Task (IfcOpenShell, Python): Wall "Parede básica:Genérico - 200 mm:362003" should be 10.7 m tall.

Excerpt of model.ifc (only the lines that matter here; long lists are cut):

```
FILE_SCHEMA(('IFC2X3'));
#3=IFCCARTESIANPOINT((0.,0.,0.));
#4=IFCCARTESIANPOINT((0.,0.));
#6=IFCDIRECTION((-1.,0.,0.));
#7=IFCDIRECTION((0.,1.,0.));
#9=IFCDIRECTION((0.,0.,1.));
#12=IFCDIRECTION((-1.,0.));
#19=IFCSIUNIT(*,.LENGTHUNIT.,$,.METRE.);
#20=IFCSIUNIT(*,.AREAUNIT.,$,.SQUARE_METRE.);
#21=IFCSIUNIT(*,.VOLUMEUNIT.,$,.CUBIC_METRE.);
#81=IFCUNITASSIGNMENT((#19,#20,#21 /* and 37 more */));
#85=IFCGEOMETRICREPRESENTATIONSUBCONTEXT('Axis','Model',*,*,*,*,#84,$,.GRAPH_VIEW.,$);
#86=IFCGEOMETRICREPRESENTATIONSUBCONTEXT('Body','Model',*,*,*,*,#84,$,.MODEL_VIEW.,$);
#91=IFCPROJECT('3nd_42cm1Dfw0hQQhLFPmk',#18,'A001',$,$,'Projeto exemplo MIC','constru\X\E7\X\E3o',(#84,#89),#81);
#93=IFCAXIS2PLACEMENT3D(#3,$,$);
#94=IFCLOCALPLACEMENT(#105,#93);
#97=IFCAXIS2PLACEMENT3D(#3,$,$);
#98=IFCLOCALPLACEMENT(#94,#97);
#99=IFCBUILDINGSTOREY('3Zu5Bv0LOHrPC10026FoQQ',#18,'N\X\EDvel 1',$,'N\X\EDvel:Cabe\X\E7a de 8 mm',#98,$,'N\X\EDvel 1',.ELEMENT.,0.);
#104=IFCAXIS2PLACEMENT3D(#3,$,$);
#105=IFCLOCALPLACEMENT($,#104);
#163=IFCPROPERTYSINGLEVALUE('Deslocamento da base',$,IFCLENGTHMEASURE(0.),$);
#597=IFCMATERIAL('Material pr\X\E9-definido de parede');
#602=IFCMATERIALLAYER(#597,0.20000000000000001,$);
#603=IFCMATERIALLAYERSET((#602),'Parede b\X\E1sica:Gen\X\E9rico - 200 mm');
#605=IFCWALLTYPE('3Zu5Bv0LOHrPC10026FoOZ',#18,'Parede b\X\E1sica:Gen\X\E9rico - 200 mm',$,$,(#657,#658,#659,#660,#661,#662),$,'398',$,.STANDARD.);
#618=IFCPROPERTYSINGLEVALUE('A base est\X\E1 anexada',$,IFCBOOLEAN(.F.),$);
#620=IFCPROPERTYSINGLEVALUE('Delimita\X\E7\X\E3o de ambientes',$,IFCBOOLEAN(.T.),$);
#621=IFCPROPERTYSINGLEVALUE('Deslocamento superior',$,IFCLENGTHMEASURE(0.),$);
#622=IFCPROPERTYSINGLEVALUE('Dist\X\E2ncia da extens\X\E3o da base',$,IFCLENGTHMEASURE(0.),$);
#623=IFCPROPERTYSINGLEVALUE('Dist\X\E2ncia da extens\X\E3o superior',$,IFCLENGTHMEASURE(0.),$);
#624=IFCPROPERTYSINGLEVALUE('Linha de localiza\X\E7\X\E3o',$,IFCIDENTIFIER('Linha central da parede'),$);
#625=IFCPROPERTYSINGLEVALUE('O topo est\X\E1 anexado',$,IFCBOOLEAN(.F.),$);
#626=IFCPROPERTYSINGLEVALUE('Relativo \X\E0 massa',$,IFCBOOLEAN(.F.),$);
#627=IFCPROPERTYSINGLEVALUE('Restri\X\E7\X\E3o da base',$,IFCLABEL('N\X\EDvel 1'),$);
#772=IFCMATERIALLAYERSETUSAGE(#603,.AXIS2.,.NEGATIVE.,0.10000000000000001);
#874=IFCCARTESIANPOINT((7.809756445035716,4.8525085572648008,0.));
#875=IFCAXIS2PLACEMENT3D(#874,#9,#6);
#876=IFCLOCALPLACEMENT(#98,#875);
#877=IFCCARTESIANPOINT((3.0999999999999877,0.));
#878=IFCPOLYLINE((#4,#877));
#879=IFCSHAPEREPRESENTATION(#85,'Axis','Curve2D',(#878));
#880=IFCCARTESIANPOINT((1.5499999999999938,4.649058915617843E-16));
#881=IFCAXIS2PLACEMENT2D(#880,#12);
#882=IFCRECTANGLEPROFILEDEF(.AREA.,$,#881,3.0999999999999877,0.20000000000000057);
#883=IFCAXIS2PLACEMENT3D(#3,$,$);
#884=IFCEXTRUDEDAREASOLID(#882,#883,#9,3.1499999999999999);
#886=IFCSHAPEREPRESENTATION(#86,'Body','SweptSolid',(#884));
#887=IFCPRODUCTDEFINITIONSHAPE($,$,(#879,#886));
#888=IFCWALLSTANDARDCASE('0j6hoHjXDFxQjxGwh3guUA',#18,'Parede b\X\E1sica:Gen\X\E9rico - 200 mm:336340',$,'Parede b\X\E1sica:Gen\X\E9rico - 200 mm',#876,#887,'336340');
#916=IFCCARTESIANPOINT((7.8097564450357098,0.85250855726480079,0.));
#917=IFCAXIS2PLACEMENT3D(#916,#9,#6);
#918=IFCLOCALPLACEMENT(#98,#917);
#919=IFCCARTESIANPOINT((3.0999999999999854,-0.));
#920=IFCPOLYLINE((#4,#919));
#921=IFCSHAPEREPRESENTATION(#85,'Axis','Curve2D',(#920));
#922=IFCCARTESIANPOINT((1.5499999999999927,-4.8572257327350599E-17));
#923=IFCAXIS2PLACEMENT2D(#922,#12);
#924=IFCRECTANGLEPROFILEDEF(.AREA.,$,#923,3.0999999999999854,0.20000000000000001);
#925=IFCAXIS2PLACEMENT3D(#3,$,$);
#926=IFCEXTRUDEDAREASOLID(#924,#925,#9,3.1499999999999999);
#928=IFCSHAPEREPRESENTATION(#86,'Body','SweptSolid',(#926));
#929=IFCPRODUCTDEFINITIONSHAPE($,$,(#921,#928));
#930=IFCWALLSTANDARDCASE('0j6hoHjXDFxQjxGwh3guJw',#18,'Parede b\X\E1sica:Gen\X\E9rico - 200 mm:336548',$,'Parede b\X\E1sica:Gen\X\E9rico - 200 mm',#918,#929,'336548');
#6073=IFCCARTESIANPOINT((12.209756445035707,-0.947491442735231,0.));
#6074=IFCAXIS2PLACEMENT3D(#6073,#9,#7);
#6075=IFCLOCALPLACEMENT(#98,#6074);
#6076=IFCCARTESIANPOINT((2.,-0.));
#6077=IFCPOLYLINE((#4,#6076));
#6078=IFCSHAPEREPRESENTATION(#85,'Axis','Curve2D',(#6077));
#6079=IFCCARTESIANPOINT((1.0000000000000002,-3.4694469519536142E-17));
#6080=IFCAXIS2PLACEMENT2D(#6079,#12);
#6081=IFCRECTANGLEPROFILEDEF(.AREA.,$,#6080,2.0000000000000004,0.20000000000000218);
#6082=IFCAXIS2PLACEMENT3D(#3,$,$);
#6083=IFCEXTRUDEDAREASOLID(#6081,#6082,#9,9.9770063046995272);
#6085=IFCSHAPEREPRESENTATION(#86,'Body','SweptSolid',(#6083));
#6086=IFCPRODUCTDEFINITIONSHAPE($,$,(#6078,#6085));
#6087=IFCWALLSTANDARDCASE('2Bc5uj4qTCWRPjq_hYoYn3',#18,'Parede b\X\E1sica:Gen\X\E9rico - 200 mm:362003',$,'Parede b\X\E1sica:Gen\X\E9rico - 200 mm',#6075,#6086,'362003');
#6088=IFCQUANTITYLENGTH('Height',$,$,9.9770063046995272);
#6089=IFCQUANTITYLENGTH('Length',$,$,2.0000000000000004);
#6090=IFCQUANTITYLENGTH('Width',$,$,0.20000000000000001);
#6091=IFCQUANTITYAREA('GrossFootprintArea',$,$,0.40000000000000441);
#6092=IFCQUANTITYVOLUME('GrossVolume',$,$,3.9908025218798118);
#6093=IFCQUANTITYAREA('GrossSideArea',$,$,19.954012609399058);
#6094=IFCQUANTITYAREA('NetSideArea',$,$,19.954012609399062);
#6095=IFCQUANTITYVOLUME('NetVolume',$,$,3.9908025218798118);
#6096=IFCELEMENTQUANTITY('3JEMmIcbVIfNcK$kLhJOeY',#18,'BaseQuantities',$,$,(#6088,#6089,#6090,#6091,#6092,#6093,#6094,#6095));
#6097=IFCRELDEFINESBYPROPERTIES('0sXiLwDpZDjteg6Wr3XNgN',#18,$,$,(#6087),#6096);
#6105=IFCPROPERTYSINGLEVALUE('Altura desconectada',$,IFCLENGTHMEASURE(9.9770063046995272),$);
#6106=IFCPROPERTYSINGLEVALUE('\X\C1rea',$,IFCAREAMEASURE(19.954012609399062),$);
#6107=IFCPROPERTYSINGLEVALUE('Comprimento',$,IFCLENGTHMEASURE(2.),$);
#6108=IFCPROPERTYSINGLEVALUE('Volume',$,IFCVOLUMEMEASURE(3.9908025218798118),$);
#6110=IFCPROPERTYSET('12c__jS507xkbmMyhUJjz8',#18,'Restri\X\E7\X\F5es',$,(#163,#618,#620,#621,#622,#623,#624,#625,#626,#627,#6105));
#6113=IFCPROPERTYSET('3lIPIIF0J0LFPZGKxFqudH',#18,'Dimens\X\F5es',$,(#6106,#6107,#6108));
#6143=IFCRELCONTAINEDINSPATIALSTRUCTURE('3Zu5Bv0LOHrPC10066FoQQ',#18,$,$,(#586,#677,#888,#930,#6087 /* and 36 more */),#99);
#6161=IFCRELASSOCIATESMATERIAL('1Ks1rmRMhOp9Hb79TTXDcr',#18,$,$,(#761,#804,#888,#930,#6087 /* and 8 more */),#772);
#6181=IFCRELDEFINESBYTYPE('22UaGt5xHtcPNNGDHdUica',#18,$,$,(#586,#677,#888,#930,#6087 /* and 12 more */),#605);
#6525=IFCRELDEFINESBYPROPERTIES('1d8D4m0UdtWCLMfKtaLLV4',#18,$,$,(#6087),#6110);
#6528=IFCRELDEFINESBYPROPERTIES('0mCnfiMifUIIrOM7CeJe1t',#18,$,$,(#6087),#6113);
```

```python
import ifcopenshell
import ifcopenshell.api.pset
import ifcopenshell.geom
import ifcopenshell.util.element
import ifcopenshell.util.representation
import ifcopenshell.util.shape
import ifcopenshell.util.unit

model = ifcopenshell.open("model.ifc")
unit_scale = ifcopenshell.util.unit.calculate_unit_scale(model)
area_scale = ifcopenshell.util.unit.calculate_unit_scale(model, "AREAUNIT")
volume_scale = ifcopenshell.util.unit.calculate_unit_scale(model, "VOLUMEUNIT")
settings = ifcopenshell.geom.settings()


def volume(element):
    """Net volume in cubic metres, openings subtracted."""
    shape = ifcopenshell.geom.create_shape(settings, element)
    return ifcopenshell.util.shape.get_volume(shape.geometry)


wall = model.by_guid("2Bc5uj4qTCWRPjq_hYoYn3")
before = volume(wall)

body = ifcopenshell.util.representation.get_representation(wall, "Model", "Body")
solid = body.Items[0]
old_height = solid.Depth
solid.Depth = 10.7 / unit_scale
after = volume(wall)
thickness = 0.2  # wall thickness in metres

# Update the stored height, areas and volumes.
qto = model.by_id(ifcopenshell.util.element.get_pset(wall, "BaseQuantities", should_inherit=False)["id"])
ifcopenshell.api.pset.edit_qto(model, qto=qto, properties={
    "Height": solid.Depth,
    "GrossVolume": ifcopenshell.util.element.get_pset(wall, "BaseQuantities", "GrossVolume") * solid.Depth / old_height,
    "GrossSideArea": ifcopenshell.util.element.get_pset(wall, "BaseQuantities", "GrossSideArea") * solid.Depth / old_height,
    "NetSideArea": after / thickness / area_scale,
    "NetVolume": after / volume_scale,
})
pset = model.by_id(ifcopenshell.util.element.get_pset(wall, "Restrições", should_inherit=False)["id"])
ifcopenshell.api.pset.edit_pset(model, pset=pset, properties={
    "Altura desconectada": model.create_entity("IfcLengthMeasure", solid.Depth),
})
pset = model.by_id(ifcopenshell.util.element.get_pset(wall, "Dimensões", should_inherit=False)["id"])
ifcopenshell.api.pset.edit_pset(model, pset=pset, properties={
    "Área": model.create_entity("IfcAreaMeasure", after / thickness / area_scale),
    "Volume": model.create_entity("IfcVolumeMeasure", after / volume_scale),
})

print(f"height {old_height:g} -> {solid.Depth:g}, volume {before:.3f} -> {after:.3f} m3")

model.write("model_edited.ifc")
```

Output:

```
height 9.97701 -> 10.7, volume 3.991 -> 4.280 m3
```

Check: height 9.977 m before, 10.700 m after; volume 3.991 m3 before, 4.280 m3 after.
